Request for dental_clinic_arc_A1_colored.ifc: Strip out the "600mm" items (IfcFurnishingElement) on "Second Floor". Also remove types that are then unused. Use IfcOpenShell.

First a look at what the model holds.

```python
import ifcopenshell
import ifcopenshell.util.element

model = ifcopenshell.open("dental_clinic_arc_A1_colored.ifc")
print(model.schema)
storey = next(s for s in model.by_type("IfcBuildingStorey") if s.Name == "Second Floor")
furniture = [e for e in ifcopenshell.util.element.get_decomposition(storey) if e.is_a("IfcFurnishingElement")]
seen = {}
for e in furniture:
    element_type = ifcopenshell.util.element.get_type(e)
    name = element_type.Name if element_type not in (None, e) else None
    seen[name] = seen.get(name, 0) + 1
for name, count in sorted(seen.items(), key=str):
    print(count, "x", name)
```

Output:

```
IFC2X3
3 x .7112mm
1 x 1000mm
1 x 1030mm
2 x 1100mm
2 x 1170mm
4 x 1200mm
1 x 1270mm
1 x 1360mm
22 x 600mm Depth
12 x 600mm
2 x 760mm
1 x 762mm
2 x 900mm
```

```python
import ifcopenshell
import ifcopenshell.api.root
import ifcopenshell.util.element

model = ifcopenshell.open("dental_clinic_arc_A1_colored.ifc")

storey = next(s for s in model.by_type("IfcBuildingStorey") if s.Name == "Second Floor")
furniture = [e for e in ifcopenshell.util.element.get_decomposition(storey) if e.is_a("IfcFurnishingElement")]
targets = [e for e in furniture if (t := ifcopenshell.util.element.get_type(e)) not in (None, e) and t.Name == "600mm"]
types = {ifcopenshell.util.element.get_type(e) for e in targets} - {None, *targets}

for e in targets:
    ifcopenshell.api.root.remove_product(model, product=e)
print(len(targets), "removed")

unused = [t for t in types if not ifcopenshell.util.element.get_types(t)]
for t in unused:
    ifcopenshell.api.root.remove_product(model, product=t)
print(len(unused), "unused types removed")

model.write("dental_clinic_arc_A1_colored_rev.ifc")
```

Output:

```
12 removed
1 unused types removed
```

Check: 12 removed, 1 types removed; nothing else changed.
